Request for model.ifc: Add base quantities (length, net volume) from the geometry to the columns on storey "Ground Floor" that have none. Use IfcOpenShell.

First a look at what the model holds.

```python
import ifcopenshell
import ifcopenshell.util.element
import ifcopenshell.util.unit

model = ifcopenshell.open("model.ifc")
print(model.schema)
for unit_type in ("LENGTHUNIT", "AREAUNIT", "VOLUMEUNIT"):
    print(unit_type, ifcopenshell.util.unit.calculate_unit_scale(model, unit_type))
storey = next(s for s in model.by_type("IfcBuildingStorey") if s.Name == "Ground Floor")
columns = [e for e in ifcopenshell.util.element.get_decomposition(storey) if e.is_a("IfcColumn")]
for e in sorted(columns, key=lambda e: e.id()):
    print(e.id(), e.is_a(), e.Name, list(ifcopenshell.util.element.get_psets(e, qtos_only=True)), sep=" | ")
```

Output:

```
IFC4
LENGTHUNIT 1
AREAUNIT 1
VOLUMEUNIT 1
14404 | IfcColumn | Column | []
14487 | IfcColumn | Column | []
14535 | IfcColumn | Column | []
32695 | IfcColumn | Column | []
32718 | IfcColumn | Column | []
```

```python
import ifcopenshell
import ifcopenshell.api.pset
import ifcopenshell.geom
import ifcopenshell.util.element
import ifcopenshell.util.shape
import ifcopenshell.util.unit

model = ifcopenshell.open("model.ifc")
unit_scale = ifcopenshell.util.unit.calculate_unit_scale(model)
volume_scale = ifcopenshell.util.unit.calculate_unit_scale(model, "VOLUMEUNIT")
settings = ifcopenshell.geom.settings()

storey = next(s for s in model.by_type("IfcBuildingStorey") if s.Name == "Ground Floor")
columns = [e for e in ifcopenshell.util.element.get_decomposition(storey) if e.is_a("IfcColumn")]

for e in sorted(columns, key=lambda e: e.id()):
    if ifcopenshell.util.element.get_psets(e, qtos_only=True, should_inherit=False):
        continue
    # Geometry comes back in metres, in the element's own axes.
    shape = ifcopenshell.geom.create_shape(settings, e)
    values = {
        "Length": ifcopenshell.util.shape.get_z(shape.geometry) / unit_scale,
        "NetVolume": ifcopenshell.util.shape.get_volume(shape.geometry) / volume_scale,
    }
    qto = ifcopenshell.api.pset.add_qto(model, product=e, name="Qto_ColumnBaseQuantities")
    ifcopenshell.api.pset.edit_qto(model, qto=qto, properties=values)
    print(e.id(), {k: round(v, 3) for k, v in values.items()})

model.write("model_v2.ifc")
```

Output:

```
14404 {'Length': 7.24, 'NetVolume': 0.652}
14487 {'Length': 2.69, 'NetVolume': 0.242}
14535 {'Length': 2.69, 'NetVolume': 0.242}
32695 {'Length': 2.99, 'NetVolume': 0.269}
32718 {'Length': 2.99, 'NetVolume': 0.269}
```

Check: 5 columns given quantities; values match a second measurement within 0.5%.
